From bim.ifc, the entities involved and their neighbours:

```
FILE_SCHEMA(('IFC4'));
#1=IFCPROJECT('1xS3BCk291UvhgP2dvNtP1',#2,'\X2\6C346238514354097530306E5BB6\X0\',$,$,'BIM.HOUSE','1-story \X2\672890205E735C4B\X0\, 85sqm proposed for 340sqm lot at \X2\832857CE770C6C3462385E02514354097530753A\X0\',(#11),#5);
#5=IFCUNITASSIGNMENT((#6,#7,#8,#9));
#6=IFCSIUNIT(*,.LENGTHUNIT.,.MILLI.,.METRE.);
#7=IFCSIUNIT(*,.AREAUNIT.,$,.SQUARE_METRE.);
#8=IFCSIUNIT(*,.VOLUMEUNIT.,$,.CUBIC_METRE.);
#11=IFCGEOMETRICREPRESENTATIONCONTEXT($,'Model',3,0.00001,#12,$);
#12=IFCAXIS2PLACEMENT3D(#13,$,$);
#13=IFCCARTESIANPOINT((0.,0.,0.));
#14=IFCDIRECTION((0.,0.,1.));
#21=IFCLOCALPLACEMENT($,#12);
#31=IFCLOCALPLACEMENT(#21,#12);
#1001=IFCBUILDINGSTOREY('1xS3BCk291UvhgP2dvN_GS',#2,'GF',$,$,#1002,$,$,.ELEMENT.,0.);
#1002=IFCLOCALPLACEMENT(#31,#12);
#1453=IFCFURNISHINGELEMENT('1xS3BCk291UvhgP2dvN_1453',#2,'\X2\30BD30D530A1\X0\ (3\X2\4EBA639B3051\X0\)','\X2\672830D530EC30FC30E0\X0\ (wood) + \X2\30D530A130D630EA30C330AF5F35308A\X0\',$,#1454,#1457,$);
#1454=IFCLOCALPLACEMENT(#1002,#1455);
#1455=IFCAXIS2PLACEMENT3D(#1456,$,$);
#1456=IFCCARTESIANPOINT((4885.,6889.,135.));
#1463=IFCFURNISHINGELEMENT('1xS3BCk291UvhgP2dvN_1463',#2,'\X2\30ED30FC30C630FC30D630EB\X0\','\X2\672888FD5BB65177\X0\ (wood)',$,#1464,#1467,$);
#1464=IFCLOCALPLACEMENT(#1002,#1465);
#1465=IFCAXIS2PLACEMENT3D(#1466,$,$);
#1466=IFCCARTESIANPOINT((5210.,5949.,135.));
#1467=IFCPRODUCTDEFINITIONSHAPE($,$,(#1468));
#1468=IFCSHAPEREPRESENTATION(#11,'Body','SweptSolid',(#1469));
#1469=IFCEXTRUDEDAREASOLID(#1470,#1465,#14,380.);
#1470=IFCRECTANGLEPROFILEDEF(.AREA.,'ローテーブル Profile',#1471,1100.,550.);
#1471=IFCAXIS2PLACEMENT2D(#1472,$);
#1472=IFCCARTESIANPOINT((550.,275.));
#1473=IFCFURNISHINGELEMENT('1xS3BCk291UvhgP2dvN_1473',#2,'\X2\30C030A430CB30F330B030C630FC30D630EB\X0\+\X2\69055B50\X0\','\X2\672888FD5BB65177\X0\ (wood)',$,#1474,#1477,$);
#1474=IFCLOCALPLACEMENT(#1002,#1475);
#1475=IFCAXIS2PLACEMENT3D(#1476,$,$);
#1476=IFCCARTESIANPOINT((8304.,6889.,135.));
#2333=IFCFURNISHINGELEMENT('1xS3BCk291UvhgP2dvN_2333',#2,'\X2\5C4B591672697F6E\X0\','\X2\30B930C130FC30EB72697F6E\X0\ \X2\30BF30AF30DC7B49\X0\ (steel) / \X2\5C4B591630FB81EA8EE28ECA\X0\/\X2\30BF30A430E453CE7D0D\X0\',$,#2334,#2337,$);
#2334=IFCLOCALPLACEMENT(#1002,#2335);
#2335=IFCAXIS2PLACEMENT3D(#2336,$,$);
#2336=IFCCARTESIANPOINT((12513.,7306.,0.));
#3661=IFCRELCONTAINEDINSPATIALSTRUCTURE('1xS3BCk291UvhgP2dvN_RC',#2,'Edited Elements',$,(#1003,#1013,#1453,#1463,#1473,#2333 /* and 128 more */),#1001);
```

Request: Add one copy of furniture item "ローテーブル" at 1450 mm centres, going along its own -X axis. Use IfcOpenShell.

```python
import ifcopenshell
import ifcopenshell.api.geometry
import ifcopenshell.api.root
import ifcopenshell.util.element
import ifcopenshell.util.placement
import ifcopenshell.util.unit

model = ifcopenshell.open("bim.ifc")
unit_scale = ifcopenshell.util.unit.calculate_unit_scale(model)


def reuse_history(source, copy):
    """copy_class also copies each property set's owner history, people and application; keep the originals."""
    for rel in copy.IsDefinedBy:
        if rel.is_a("IfcRelDefinesByProperties") and (history := rel.RelatingPropertyDefinition.OwnerHistory):
            rel.RelatingPropertyDefinition.OwnerHistory = source.OwnerHistory
            ifcopenshell.util.element.remove_deep2(model, history)


source = model.by_id(1463)
base = ifcopenshell.util.placement.get_local_placement(source.ObjectPlacement)
step = -base[:3, 0] * 1.45 / unit_scale

for i in range(1, 2):
    copy = ifcopenshell.api.root.copy_class(model, product=source)
    copy.Representation = ifcopenshell.util.element.copy_deep(
        model, source.Representation, exclude=["IfcGeometricRepresentationContext", "IfcRepresentationMap"]
    )
    reuse_history(source, copy)
    matrix = base.copy()
    matrix[:3, 3] += i * step
    print("added at", matrix[:3, 3].round(3) + 0.0)
    ifcopenshell.api.geometry.edit_object_placement(model, product=copy, matrix=matrix, is_si=False)

model.write("bim_updated.ifc")
```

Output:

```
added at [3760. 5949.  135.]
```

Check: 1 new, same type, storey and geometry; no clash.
